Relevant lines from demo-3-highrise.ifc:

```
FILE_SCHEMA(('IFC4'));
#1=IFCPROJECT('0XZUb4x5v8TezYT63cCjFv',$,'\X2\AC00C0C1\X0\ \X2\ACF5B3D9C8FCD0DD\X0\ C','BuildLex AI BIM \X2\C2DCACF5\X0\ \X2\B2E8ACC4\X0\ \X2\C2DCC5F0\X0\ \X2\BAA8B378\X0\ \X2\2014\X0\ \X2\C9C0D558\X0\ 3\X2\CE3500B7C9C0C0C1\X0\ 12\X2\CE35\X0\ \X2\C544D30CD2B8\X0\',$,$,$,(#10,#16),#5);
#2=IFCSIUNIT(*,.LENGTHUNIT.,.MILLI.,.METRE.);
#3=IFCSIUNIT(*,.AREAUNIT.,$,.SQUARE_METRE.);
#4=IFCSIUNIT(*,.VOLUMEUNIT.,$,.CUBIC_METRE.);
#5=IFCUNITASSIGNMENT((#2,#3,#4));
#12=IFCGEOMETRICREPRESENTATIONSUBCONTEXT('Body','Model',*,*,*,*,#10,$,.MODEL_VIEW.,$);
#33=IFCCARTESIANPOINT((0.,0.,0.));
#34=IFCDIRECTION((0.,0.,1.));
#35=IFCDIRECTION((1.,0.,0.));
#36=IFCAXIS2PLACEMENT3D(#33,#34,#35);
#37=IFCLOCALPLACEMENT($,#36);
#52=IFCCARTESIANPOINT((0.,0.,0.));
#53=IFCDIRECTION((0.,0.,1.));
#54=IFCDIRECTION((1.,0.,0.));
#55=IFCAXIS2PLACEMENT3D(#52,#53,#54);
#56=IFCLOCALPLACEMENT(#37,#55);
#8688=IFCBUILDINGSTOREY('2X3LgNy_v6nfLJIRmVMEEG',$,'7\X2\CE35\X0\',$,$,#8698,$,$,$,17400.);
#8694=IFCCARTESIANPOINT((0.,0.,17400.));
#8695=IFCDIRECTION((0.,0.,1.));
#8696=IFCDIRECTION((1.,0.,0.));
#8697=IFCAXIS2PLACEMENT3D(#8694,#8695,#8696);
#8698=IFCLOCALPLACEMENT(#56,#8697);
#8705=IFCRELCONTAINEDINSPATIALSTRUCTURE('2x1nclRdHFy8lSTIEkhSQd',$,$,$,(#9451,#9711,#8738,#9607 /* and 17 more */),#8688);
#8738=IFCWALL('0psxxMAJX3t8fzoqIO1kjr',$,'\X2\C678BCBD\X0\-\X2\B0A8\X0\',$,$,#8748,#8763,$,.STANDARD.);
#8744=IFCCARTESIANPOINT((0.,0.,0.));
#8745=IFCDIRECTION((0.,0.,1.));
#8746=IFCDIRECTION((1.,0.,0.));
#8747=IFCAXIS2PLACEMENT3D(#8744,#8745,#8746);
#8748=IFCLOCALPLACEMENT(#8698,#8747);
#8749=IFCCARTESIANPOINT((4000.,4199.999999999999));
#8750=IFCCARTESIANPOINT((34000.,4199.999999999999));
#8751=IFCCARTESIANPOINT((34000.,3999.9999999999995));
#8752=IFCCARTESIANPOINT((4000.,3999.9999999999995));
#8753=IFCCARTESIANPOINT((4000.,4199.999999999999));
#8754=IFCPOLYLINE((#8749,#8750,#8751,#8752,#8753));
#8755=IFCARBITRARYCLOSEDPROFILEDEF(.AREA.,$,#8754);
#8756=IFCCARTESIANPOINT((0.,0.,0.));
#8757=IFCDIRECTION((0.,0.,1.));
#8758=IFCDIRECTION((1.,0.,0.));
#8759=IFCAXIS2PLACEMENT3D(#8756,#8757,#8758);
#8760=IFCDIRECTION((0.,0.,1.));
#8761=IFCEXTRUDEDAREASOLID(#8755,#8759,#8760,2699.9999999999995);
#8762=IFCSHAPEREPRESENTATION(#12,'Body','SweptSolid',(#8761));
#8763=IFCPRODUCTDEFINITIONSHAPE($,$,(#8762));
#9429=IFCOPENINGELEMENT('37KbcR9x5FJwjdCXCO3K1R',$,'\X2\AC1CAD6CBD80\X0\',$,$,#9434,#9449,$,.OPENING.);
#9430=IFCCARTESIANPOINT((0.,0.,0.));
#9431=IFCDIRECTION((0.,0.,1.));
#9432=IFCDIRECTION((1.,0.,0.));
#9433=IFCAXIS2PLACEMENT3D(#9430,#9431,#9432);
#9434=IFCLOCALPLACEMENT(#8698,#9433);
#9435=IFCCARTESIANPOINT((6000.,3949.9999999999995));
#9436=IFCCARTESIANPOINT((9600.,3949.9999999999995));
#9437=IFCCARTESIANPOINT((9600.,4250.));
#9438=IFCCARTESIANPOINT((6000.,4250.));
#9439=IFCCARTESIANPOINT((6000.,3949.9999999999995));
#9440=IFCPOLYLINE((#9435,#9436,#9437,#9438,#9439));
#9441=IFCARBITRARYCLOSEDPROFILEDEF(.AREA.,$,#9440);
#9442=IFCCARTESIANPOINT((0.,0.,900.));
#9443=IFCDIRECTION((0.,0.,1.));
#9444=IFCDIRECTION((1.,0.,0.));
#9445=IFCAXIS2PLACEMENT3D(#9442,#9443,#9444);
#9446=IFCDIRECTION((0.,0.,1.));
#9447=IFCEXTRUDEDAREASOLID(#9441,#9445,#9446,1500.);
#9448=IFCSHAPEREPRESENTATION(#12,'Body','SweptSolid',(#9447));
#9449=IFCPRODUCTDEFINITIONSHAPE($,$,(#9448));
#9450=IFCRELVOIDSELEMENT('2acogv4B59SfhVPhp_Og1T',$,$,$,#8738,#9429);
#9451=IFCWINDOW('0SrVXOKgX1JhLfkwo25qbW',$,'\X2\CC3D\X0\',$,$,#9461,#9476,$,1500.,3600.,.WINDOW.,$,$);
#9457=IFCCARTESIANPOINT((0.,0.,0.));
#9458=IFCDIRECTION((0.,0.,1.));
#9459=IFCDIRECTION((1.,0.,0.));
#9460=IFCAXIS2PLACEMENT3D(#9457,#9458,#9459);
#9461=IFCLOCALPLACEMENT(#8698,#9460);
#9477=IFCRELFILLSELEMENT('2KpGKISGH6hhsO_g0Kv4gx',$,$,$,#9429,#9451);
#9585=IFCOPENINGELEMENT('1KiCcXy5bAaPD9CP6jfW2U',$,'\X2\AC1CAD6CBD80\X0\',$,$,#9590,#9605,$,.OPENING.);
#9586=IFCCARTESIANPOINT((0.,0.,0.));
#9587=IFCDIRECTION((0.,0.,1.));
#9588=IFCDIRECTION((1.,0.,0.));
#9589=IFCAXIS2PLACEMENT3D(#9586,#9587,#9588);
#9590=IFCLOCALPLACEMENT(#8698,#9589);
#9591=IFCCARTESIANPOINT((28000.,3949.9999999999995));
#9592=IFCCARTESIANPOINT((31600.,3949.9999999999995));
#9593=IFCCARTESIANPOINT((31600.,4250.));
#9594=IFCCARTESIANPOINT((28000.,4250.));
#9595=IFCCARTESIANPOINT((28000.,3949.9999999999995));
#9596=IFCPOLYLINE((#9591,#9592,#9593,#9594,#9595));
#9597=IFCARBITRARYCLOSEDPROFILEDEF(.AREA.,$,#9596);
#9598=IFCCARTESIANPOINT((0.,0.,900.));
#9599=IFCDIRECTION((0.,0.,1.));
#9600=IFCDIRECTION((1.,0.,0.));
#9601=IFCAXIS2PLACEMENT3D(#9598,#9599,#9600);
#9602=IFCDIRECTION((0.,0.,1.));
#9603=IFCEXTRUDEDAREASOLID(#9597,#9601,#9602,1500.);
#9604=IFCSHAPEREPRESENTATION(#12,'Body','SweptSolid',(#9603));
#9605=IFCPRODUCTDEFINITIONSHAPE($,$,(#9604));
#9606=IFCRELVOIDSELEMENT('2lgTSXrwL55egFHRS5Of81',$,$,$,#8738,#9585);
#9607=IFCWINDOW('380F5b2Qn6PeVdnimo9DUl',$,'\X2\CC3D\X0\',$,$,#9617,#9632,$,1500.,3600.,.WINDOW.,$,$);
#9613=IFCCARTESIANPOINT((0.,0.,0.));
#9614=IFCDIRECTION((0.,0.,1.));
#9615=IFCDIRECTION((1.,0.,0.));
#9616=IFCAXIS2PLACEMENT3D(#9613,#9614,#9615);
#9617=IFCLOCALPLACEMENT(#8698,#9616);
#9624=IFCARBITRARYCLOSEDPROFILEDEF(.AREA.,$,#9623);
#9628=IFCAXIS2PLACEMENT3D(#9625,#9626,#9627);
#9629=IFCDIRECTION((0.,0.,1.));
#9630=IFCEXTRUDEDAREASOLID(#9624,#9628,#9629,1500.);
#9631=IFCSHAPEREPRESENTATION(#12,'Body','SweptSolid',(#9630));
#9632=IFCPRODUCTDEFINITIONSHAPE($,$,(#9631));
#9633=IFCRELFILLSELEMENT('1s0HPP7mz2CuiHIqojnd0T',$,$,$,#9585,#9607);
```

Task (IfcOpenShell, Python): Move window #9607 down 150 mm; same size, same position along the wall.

```python
import numpy as np
import ifcopenshell
import ifcopenshell.api.geometry
import ifcopenshell.util.placement
import ifcopenshell.util.unit

model = ifcopenshell.open("demo-3-highrise.ifc")
unit_scale = ifcopenshell.util.unit.calculate_unit_scale(model)

window = model.by_guid("380F5b2Qn6PeVdnimo9DUl")
opening = window.FillsVoids[0].RelatingOpeningElement
dz = -150.0

shift = np.array([0.0, 0.0, dz])
# The window is not placed relative to its opening, so move both.
for product in (opening, window):
    matrix = ifcopenshell.util.placement.get_local_placement(product.ObjectPlacement)
    matrix[:3, 3] += shift
    ifcopenshell.api.geometry.edit_object_placement(model, product=product, matrix=matrix, is_si=False)

print(f"moved by {dz * unit_scale:+.3f} m")

model.write("demo-3-highrise_edited.ifc")
```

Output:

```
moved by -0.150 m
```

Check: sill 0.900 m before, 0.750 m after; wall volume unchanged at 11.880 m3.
